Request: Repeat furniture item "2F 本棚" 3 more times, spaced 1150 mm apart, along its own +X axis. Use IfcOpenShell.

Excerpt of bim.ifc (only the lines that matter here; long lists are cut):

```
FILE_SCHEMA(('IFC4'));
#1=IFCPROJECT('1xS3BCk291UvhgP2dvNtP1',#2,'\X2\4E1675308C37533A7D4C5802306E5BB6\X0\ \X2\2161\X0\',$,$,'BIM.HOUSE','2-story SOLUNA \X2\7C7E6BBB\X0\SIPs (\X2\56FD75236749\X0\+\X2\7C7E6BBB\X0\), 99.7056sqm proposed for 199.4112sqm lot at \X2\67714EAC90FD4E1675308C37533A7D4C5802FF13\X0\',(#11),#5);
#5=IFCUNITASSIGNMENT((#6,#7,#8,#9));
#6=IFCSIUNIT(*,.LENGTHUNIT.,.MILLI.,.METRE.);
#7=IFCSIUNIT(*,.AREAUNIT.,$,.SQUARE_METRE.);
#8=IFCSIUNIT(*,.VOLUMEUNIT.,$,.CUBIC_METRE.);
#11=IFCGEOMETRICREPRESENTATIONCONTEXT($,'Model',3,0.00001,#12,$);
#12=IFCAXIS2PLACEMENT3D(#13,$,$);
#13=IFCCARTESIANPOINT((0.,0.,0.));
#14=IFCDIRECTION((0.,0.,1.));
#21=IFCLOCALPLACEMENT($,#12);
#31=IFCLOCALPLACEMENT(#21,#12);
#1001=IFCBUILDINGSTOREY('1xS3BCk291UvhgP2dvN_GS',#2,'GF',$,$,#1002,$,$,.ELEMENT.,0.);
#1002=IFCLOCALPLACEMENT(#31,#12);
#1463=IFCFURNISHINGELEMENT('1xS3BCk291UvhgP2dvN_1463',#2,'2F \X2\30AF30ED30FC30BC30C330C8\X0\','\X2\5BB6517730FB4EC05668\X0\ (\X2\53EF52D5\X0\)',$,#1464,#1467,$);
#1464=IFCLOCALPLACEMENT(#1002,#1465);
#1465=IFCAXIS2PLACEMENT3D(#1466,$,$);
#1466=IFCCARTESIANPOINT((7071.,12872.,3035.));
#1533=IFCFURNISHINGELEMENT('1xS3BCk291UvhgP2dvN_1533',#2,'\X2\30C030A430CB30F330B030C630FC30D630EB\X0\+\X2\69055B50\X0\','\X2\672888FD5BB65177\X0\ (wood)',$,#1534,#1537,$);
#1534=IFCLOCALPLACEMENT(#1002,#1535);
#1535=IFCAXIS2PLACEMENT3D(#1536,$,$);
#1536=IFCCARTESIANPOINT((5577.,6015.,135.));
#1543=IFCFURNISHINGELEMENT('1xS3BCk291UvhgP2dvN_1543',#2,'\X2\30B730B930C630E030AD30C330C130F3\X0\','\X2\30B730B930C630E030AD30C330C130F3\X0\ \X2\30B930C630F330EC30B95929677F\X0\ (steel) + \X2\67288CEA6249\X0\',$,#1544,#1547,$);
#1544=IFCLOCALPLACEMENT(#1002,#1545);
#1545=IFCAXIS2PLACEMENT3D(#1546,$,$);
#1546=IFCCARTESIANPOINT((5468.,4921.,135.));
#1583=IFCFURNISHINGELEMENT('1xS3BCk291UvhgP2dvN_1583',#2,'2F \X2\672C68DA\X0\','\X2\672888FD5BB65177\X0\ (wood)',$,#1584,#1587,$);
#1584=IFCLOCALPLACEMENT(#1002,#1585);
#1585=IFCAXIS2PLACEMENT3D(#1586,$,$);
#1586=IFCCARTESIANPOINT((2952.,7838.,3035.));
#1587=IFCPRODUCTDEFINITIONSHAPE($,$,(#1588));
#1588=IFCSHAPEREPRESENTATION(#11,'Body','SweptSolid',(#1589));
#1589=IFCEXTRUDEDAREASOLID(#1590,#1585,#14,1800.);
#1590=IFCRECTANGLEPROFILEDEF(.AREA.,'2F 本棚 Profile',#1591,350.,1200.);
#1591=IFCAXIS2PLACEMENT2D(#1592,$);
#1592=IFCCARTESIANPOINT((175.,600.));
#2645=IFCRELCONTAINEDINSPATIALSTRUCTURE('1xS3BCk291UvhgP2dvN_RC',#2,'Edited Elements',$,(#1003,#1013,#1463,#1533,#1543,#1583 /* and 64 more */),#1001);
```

```python
import ifcopenshell
import ifcopenshell.api.geometry
import ifcopenshell.api.root
import ifcopenshell.util.element
import ifcopenshell.util.placement

model = ifcopenshell.open("bim.ifc")


def reuse_history(source, copy):
    """copy_class also copies each property set's owner history, people and application; keep the originals."""
    for rel in copy.IsDefinedBy:
        if rel.is_a("IfcRelDefinesByProperties") and (history := rel.RelatingPropertyDefinition.OwnerHistory):
            rel.RelatingPropertyDefinition.OwnerHistory = source.OwnerHistory
            ifcopenshell.util.element.remove_deep2(model, history)


source = model.by_guid("1xS3BCk291UvhgP2dvN_1583")
base = ifcopenshell.util.placement.get_local_placement(source.ObjectPlacement)
step = base[:3, 0] * 1150.0

for i in range(1, 4):
    copy = ifcopenshell.api.root.copy_class(model, product=source)
    copy.Representation = ifcopenshell.util.element.copy_deep(
        model, source.Representation, exclude=["IfcGeometricRepresentationContext", "IfcRepresentationMap"]
    )
    reuse_history(source, copy)
    matrix = base.copy()
    matrix[:3, 3] += i * step
    print("added at", matrix[:3, 3].round(3) + 0.0)
    ifcopenshell.api.geometry.edit_object_placement(model, product=copy, matrix=matrix, is_si=False)

model.write("bim_rev.ifc")
```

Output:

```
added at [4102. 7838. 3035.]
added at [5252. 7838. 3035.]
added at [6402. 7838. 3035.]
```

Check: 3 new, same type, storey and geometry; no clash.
